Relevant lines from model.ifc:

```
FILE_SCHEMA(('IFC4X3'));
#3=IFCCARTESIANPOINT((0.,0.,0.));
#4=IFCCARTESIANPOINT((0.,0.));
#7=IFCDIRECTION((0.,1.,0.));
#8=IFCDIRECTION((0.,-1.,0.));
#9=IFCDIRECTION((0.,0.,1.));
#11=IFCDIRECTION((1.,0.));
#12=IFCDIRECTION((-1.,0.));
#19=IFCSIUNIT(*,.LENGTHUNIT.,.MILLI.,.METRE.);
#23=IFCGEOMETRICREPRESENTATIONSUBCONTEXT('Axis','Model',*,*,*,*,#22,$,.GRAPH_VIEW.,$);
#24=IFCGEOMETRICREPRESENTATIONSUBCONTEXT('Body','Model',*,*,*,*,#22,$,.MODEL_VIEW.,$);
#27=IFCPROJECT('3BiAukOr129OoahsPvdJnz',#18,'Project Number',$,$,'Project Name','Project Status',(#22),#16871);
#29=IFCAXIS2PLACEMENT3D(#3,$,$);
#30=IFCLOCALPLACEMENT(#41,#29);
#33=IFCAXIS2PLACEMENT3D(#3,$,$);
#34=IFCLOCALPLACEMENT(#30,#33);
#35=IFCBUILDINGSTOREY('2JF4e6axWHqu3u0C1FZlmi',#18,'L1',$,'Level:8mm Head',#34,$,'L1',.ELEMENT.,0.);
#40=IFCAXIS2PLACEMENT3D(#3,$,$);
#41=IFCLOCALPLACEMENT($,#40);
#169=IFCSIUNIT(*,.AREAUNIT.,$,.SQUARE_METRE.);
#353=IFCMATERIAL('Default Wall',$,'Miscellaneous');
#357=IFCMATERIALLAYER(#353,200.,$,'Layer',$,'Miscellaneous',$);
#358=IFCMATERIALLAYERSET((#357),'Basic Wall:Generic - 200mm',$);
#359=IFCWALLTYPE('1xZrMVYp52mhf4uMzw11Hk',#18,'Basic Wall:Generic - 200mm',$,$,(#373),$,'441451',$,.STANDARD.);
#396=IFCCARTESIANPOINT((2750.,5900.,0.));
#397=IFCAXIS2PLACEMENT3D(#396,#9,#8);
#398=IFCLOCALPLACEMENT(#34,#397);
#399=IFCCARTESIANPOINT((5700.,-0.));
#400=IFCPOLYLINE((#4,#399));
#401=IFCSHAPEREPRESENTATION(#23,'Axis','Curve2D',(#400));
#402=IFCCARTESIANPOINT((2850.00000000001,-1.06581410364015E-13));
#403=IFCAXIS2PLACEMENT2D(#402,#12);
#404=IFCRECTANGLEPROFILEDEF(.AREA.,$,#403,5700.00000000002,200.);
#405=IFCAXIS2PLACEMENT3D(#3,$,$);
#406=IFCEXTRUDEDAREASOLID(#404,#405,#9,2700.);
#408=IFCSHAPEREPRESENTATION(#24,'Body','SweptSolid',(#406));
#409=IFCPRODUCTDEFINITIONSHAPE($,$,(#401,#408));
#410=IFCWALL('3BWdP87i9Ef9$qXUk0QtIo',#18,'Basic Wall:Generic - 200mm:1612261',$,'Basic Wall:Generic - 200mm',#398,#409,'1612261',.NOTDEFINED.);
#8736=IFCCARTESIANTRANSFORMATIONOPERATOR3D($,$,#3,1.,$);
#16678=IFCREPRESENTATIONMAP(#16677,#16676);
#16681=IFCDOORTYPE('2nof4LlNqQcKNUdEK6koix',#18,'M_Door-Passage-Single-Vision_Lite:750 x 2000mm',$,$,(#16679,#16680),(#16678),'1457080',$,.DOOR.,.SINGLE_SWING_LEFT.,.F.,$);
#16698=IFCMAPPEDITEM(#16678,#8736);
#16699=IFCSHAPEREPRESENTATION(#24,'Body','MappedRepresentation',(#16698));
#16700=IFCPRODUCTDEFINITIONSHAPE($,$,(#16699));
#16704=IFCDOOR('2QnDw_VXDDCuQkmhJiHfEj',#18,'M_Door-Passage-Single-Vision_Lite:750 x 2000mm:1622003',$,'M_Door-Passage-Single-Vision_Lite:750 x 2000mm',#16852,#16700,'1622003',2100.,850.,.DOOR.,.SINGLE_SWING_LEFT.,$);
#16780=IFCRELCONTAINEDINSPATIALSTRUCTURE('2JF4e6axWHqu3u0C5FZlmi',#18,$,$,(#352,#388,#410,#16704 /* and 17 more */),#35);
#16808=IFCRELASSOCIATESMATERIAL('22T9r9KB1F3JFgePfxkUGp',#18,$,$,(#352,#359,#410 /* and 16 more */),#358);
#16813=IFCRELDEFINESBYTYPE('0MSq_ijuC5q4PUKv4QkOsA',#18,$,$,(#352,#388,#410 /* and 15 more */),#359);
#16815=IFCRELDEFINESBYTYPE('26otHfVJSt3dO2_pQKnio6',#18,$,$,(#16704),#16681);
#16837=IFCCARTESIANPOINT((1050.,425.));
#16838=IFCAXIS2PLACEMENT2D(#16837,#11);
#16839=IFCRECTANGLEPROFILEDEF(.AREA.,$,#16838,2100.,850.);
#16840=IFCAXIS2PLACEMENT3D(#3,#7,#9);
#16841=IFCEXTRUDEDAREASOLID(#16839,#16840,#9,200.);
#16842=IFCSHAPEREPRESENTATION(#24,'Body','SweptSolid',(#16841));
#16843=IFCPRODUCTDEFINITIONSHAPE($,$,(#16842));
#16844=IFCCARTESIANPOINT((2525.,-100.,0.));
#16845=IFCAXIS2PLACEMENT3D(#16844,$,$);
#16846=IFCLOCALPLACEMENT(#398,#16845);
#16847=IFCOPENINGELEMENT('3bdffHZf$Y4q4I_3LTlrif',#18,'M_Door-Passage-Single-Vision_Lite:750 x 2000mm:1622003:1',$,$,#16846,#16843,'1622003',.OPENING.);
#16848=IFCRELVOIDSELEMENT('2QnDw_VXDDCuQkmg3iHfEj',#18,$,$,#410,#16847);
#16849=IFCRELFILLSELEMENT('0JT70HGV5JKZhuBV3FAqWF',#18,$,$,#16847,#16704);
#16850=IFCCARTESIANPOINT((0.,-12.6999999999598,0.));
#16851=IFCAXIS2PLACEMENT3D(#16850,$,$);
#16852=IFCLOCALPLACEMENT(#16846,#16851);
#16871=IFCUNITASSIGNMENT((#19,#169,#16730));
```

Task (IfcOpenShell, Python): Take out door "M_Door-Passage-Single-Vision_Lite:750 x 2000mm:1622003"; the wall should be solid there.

```python
import ifcopenshell
import ifcopenshell.api.feature
import ifcopenshell.api.root
import ifcopenshell.geom
import ifcopenshell.util.shape

model = ifcopenshell.open("model.ifc")
settings = ifcopenshell.geom.settings()


def volume(element):
    """Net volume in cubic metres, openings subtracted."""
    shape = ifcopenshell.geom.create_shape(settings, element)
    return ifcopenshell.util.shape.get_volume(shape.geometry)


door = model.by_guid("2QnDw_VXDDCuQkmhJiHfEj")
opening = door.FillsVoids[0].RelatingOpeningElement
wall = opening.VoidsElements[0].RelatingBuildingElement
before = volume(wall)

ifcopenshell.api.root.remove_product(model, product=door)
ifcopenshell.api.feature.remove_feature(model, feature=opening)

after = volume(wall)

print(f"wall volume {before:.3f} -> {after:.3f} m3")

model.write("model_rev.ifc")
```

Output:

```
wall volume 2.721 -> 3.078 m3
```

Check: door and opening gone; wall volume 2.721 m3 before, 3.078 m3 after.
